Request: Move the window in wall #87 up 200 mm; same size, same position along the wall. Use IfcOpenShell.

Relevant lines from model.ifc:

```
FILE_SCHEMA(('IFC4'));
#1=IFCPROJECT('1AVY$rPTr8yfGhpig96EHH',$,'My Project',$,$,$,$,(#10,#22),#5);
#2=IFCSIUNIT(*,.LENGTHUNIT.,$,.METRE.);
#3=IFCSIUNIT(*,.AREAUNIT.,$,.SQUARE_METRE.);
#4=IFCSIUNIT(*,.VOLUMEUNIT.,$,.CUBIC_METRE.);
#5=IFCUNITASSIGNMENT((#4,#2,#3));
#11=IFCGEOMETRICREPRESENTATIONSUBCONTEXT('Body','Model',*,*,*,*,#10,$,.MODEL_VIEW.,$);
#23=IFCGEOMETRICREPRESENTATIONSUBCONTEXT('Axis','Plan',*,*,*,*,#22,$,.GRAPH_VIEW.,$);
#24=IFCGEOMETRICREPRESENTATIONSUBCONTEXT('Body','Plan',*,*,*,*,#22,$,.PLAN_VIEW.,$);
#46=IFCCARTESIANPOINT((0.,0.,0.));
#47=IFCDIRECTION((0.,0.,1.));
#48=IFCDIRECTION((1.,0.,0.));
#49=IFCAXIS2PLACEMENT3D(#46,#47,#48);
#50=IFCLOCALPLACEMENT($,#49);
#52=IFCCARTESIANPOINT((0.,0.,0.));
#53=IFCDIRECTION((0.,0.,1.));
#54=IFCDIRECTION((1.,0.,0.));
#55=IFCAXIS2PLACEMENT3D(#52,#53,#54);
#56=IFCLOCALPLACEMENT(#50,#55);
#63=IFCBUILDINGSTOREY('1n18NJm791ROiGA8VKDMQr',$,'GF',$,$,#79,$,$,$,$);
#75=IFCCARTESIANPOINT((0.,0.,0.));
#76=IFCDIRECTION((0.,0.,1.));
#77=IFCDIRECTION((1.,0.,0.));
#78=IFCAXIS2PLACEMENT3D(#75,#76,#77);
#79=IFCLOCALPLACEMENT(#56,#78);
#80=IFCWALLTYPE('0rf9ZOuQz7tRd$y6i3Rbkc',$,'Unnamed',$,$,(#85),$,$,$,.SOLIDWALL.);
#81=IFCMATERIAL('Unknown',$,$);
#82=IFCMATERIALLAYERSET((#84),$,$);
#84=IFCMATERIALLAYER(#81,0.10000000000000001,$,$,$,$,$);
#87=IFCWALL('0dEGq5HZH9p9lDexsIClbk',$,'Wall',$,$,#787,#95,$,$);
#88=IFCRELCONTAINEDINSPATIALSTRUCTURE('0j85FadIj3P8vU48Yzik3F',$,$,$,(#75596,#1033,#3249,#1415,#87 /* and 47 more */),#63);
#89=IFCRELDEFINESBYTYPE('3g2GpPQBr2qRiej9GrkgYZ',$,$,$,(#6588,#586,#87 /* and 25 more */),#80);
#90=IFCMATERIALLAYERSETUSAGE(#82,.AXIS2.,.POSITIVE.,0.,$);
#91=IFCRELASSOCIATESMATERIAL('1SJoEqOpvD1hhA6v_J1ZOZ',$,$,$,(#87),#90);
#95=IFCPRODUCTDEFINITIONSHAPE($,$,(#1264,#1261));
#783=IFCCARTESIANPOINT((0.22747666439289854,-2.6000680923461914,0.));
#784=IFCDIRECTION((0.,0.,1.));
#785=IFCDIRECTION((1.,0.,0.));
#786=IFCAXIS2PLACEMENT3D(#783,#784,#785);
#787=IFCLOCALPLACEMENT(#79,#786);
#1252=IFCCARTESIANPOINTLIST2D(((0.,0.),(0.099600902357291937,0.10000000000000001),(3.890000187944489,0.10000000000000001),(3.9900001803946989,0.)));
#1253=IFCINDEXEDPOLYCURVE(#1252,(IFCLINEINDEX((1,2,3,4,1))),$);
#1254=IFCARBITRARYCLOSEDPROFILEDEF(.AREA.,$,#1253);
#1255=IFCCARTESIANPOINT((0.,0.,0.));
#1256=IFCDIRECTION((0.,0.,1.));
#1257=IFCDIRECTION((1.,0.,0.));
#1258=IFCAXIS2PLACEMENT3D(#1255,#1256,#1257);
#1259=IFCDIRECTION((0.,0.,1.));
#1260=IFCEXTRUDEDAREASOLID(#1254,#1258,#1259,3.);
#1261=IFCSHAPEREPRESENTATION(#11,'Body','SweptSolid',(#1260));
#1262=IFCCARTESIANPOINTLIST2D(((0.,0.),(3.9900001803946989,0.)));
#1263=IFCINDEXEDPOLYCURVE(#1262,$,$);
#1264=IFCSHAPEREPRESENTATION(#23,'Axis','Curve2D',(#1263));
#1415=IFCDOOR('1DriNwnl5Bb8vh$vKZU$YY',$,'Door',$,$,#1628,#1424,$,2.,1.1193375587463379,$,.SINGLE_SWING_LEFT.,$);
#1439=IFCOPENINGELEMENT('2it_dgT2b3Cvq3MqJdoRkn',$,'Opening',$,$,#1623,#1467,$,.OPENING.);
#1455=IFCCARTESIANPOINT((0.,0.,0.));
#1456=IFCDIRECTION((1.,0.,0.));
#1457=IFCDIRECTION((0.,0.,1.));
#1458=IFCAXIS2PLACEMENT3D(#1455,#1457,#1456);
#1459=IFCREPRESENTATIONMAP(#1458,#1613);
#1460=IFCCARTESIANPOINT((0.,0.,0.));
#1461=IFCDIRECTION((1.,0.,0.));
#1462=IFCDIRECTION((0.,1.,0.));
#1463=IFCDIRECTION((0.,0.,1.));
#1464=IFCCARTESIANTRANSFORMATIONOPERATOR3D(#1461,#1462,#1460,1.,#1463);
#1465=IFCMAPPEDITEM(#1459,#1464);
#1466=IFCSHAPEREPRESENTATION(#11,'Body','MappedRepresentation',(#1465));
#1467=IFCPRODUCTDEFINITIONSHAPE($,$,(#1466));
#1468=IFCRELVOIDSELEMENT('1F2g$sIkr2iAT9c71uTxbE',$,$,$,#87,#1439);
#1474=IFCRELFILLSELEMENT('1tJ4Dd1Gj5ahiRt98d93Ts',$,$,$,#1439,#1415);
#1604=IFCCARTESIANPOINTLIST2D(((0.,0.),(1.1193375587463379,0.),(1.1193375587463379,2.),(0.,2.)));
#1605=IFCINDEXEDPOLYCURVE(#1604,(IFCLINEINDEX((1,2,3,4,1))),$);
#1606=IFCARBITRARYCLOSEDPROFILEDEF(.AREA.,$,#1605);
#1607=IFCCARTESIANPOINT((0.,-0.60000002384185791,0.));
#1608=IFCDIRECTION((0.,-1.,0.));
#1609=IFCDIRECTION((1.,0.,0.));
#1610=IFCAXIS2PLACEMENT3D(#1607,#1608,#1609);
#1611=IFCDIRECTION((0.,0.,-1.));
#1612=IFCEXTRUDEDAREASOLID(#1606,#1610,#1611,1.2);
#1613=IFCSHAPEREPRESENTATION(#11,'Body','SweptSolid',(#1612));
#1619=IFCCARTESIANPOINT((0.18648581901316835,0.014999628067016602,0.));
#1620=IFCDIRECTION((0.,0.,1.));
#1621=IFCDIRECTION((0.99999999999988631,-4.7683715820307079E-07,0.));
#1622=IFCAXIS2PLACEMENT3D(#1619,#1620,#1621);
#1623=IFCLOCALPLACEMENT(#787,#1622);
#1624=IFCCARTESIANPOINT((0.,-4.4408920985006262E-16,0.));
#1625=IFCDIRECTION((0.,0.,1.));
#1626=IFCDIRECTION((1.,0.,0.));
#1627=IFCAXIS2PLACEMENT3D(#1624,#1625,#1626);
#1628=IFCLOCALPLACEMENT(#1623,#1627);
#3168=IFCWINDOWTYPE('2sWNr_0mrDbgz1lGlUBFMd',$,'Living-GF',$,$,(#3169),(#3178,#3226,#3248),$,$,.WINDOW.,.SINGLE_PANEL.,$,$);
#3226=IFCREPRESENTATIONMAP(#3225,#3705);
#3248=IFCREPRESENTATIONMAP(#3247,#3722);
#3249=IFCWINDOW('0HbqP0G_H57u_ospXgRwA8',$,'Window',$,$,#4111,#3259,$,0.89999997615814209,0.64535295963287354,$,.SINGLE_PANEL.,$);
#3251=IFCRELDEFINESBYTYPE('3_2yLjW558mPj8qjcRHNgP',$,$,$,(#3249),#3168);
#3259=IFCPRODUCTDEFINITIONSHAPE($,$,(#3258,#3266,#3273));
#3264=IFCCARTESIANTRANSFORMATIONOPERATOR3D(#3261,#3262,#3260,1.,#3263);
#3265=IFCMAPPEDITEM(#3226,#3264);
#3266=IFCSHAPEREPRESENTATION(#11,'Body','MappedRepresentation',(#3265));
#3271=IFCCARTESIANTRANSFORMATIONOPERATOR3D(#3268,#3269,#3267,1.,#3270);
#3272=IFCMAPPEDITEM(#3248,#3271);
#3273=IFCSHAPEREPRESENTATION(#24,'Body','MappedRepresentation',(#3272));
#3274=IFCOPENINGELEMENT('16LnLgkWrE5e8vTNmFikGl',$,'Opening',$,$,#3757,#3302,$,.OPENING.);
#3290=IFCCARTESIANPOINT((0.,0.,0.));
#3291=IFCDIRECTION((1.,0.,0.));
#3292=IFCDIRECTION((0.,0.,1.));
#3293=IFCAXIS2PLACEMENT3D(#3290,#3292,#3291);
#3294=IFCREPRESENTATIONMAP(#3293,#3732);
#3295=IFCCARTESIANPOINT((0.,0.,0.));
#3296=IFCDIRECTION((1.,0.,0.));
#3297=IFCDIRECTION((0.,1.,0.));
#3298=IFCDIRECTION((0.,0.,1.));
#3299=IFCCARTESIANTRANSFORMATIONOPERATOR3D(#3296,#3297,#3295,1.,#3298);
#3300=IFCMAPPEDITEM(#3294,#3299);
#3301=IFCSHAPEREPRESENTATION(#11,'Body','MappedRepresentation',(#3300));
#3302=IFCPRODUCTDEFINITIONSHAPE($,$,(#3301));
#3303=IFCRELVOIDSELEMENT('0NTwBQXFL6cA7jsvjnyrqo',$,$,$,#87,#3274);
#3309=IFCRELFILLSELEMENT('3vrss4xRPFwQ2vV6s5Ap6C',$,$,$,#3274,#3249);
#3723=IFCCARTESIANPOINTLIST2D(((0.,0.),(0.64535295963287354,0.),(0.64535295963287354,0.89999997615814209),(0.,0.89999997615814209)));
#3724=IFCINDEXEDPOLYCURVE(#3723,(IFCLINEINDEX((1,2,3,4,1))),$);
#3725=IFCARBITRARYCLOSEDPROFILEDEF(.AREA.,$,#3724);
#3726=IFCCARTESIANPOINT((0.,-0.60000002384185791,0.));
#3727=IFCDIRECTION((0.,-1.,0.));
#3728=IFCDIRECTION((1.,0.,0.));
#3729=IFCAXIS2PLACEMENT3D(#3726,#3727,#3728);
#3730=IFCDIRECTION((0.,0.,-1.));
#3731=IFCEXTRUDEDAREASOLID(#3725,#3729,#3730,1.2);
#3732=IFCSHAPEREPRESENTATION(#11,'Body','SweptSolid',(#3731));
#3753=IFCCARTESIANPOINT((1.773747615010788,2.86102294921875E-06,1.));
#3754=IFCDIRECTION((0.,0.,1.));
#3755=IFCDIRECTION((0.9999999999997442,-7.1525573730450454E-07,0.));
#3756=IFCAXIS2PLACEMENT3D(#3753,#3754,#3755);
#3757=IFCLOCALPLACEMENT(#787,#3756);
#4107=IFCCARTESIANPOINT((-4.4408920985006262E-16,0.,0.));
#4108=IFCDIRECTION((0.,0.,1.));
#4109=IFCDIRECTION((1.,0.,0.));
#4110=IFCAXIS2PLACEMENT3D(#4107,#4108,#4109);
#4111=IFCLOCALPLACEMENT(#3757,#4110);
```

```python
import numpy as np
import ifcopenshell
import ifcopenshell.api.geometry
import ifcopenshell.util.placement
import ifcopenshell.util.unit

model = ifcopenshell.open("model.ifc")
unit_scale = ifcopenshell.util.unit.calculate_unit_scale(model)

window = model.by_id(3249)
opening = window.FillsVoids[0].RelatingOpeningElement
dz = 0.2

shift = np.array([0.0, 0.0, dz])
# The window is placed relative to its opening, so it follows when the opening moves.
matrix = ifcopenshell.util.placement.get_local_placement(opening.ObjectPlacement)
matrix[:3, 3] += shift
ifcopenshell.api.geometry.edit_object_placement(
    model, product=opening, matrix=matrix, is_si=False, should_transform_children=True
)

print(f"moved by {dz * unit_scale:+.3f} m")

model.write("model_edited.ifc")
```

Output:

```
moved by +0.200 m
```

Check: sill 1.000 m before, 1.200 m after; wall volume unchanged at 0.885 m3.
